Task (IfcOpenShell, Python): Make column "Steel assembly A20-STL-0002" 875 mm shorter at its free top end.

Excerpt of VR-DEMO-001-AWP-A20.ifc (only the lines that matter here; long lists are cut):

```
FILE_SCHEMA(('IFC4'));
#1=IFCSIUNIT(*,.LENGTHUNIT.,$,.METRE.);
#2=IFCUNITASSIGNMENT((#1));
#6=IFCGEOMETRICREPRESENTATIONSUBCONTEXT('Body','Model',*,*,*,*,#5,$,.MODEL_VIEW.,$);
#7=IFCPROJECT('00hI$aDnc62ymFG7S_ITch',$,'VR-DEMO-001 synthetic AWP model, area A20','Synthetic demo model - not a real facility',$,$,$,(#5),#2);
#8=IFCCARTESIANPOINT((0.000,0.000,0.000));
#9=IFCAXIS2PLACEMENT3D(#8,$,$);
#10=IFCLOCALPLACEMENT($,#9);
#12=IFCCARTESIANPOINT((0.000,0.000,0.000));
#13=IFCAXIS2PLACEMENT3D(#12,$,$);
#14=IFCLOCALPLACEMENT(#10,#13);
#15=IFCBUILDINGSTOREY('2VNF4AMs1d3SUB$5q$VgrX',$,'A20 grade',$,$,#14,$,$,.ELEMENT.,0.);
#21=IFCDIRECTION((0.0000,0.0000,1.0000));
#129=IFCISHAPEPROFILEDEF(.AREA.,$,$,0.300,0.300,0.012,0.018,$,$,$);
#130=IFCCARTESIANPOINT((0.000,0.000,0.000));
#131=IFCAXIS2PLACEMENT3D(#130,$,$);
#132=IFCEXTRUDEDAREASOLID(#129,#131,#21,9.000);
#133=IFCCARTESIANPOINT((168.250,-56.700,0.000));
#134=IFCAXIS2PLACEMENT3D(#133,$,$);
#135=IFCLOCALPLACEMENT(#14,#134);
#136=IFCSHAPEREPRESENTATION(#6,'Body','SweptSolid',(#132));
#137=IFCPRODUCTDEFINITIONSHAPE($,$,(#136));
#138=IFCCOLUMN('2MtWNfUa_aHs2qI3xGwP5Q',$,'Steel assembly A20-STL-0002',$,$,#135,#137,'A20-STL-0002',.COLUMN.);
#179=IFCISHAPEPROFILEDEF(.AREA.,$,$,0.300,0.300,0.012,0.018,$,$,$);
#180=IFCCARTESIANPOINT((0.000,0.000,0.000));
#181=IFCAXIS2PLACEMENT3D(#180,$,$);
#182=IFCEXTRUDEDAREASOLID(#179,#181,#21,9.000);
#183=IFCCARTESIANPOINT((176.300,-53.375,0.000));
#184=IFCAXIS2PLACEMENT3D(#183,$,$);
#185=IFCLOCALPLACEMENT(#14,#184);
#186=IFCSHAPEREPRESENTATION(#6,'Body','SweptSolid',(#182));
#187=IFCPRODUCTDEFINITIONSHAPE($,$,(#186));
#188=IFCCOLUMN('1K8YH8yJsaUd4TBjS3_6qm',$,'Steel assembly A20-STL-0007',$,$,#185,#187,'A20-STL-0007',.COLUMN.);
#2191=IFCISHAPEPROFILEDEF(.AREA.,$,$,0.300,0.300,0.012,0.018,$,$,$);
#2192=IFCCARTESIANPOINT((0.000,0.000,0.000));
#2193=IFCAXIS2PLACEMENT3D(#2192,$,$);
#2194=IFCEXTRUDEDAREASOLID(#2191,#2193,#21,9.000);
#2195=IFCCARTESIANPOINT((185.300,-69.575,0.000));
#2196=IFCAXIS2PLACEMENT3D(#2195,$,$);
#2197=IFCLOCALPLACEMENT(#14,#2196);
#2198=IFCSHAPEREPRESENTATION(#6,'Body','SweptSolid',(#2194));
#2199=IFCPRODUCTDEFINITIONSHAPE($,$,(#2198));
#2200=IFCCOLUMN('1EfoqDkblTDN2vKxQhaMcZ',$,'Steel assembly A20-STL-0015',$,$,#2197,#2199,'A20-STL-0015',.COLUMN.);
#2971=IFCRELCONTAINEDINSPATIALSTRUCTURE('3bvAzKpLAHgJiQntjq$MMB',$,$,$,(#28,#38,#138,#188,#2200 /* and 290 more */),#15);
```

```python
import ifcopenshell
import ifcopenshell.util.representation
import ifcopenshell.util.unit

model = ifcopenshell.open("VR-DEMO-001-AWP-A20.ifc")
unit_scale = ifcopenshell.util.unit.calculate_unit_scale(model)

member = model.by_guid("2MtWNfUa_aHs2qI3xGwP5Q")
change = -0.875 / unit_scale

# The extrusion runs towards the end named, so only its depth changes.
body = ifcopenshell.util.representation.get_representation(member, "Model", "Body")
solid = body.Items[0]
old_length = solid.Depth
solid.Depth += change

print(f"length {old_length:g} -> {solid.Depth:g}")

model.write("VR-DEMO-001-AWP-A20_v2.ifc")
```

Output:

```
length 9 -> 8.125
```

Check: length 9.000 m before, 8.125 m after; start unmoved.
